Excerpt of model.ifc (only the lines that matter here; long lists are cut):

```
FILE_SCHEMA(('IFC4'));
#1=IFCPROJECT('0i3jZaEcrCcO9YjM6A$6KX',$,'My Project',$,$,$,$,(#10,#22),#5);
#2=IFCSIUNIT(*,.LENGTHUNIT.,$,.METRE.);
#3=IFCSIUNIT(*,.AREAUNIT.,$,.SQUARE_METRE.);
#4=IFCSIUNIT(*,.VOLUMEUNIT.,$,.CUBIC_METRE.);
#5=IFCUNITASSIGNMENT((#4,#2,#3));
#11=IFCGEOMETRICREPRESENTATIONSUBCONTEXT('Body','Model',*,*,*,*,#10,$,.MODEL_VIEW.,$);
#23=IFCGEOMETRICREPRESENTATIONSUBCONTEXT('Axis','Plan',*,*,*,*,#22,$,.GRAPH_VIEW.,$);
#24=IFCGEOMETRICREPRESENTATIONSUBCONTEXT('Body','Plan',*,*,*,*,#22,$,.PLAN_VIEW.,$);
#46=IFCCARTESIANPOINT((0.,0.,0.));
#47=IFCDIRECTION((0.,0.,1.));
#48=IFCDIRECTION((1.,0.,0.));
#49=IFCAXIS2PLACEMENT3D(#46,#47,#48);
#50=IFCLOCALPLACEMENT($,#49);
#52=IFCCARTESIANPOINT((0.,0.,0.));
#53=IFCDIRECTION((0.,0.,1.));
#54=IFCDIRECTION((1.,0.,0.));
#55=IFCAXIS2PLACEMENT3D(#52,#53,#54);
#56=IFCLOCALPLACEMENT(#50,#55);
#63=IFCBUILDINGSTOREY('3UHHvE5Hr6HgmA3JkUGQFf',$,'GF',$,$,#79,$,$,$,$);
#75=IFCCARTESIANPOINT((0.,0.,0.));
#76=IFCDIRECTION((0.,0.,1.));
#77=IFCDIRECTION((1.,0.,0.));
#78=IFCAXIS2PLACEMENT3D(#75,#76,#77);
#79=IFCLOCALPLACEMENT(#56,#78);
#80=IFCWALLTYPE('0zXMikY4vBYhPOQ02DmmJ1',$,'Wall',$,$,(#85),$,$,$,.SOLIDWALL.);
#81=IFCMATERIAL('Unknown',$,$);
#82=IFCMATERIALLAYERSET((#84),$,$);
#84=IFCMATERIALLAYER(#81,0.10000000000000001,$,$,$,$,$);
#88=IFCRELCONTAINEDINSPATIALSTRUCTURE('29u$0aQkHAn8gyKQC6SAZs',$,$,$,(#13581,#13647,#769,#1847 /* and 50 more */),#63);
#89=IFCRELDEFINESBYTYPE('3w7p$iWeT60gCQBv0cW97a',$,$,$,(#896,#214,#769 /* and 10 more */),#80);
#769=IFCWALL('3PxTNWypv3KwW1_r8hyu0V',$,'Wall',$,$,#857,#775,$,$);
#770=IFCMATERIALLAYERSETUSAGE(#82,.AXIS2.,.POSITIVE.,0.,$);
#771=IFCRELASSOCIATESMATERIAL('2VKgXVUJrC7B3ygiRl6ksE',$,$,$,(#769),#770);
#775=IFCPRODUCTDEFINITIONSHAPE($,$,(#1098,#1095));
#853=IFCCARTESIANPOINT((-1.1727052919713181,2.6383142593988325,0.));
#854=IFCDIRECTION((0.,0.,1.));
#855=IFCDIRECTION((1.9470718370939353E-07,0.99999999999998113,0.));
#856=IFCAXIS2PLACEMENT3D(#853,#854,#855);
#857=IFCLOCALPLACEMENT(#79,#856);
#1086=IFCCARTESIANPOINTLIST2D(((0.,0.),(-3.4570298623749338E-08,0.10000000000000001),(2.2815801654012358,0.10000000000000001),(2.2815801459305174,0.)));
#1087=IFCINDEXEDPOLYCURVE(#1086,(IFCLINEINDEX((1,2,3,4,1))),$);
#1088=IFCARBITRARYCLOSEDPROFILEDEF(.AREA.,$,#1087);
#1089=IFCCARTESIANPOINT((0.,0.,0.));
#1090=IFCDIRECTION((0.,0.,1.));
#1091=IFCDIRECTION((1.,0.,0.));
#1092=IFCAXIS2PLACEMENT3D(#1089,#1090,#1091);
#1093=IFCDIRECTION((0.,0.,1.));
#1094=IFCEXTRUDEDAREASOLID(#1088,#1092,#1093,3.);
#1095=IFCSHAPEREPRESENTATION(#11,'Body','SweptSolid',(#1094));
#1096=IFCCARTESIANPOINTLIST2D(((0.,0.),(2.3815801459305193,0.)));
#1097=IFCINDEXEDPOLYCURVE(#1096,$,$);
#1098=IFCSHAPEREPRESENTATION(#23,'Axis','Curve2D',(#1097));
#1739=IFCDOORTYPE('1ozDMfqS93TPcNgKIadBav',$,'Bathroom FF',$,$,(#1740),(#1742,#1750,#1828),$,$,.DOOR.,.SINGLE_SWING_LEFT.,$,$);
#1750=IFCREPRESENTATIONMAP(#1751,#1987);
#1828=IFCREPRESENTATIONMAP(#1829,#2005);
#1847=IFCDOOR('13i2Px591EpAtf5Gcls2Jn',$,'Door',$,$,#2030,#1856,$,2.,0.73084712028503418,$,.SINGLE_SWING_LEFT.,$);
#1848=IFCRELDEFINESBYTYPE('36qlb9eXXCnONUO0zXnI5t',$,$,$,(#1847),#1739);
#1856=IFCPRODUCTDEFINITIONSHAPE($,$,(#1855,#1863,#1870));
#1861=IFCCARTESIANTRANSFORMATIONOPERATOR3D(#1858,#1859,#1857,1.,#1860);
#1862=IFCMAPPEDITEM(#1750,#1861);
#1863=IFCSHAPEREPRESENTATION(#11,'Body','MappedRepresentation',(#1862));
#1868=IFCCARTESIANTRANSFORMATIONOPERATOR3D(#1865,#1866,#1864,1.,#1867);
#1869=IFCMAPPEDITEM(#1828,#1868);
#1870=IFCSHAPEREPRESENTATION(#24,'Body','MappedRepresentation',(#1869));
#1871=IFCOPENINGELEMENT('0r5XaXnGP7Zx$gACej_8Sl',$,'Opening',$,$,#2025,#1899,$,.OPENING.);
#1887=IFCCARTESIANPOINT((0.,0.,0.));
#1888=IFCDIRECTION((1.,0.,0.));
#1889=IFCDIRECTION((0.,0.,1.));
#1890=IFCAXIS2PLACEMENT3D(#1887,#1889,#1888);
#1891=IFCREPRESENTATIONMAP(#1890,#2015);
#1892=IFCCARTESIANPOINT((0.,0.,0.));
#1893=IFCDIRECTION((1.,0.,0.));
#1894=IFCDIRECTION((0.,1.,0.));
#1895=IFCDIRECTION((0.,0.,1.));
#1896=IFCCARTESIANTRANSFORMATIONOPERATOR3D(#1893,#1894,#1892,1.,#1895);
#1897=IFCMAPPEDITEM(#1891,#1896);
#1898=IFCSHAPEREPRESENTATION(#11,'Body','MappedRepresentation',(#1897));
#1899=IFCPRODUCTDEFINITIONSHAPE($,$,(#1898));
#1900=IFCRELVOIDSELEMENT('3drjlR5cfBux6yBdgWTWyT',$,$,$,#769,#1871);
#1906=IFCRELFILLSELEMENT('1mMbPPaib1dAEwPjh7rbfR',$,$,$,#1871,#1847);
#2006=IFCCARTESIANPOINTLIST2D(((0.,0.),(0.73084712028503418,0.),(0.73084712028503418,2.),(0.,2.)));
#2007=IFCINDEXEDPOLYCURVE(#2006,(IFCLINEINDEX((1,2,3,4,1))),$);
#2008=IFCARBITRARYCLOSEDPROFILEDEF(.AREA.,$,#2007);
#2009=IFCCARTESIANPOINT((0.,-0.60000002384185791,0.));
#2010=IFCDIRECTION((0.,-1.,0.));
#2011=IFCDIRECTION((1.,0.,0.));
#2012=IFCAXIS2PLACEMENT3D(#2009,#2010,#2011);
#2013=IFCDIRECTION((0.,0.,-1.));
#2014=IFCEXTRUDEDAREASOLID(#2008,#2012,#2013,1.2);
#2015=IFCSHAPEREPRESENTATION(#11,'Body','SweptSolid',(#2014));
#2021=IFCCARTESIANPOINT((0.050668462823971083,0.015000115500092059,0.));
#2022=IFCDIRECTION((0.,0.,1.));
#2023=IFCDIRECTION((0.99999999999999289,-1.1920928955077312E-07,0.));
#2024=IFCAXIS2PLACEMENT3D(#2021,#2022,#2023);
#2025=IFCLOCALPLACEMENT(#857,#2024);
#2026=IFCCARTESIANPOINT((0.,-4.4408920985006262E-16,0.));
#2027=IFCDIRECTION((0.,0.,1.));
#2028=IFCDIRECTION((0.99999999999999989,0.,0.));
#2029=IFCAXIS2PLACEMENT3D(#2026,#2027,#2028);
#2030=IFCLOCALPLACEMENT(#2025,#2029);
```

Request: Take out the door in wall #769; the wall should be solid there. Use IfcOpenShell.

```python
import ifcopenshell
import ifcopenshell.api.feature
import ifcopenshell.api.root
import ifcopenshell.geom
import ifcopenshell.util.shape

model = ifcopenshell.open("model.ifc")
settings = ifcopenshell.geom.settings()


def volume(element):
    """Net volume in cubic metres, openings subtracted."""
    shape = ifcopenshell.geom.create_shape(settings, element)
    return ifcopenshell.util.shape.get_volume(shape.geometry)


door = model.by_guid("13i2Px591EpAtf5Gcls2Jn")
opening = door.FillsVoids[0].RelatingOpeningElement
wall = opening.VoidsElements[0].RelatingBuildingElement
before = volume(wall)

ifcopenshell.api.root.remove_product(model, product=door)
ifcopenshell.api.feature.remove_feature(model, feature=opening)

after = volume(wall)

print(f"wall volume {before:.3f} -> {after:.3f} m3")

model.write("model_rev.ifc")
```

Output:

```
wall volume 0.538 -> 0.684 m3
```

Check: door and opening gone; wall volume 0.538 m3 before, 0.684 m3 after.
